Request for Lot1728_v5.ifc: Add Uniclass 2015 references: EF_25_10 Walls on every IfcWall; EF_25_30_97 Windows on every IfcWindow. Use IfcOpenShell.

First a look at what the model holds.

```python
import ifcopenshell

model = ifcopenshell.open("Lot1728_v5.ifc")
print(model.schema)
print("classifications:", [c.Name for c in model.by_type("IfcClassification")])
for ifc_class in ("IfcDoor", "IfcRoof", "IfcStair", "IfcWall", "IfcWindow"):
    print(ifc_class, len(model.by_type(ifc_class)))
```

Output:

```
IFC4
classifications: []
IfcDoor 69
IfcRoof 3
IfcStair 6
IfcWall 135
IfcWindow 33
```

```python
import ifcopenshell
import ifcopenshell.api.classification

model = ifcopenshell.open("Lot1728_v5.ifc")

system = ifcopenshell.api.classification.add_classification(model, classification="Uniclass 2015")

codes = {
    "IfcWall": ("EF_25_10", "Walls"),
    "IfcWindow": ("EF_25_30_97", "Windows"),
}
for ifc_class, (code, name) in codes.items():
    products = model.by_type(ifc_class)
    ifcopenshell.api.classification.add_reference(
        model, products=products, classification=system, identification=code, name=name
    )
    print(code, len(products))

model.write("Lot1728_v5-out.ifc")
```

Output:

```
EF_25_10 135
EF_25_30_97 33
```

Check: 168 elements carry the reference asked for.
